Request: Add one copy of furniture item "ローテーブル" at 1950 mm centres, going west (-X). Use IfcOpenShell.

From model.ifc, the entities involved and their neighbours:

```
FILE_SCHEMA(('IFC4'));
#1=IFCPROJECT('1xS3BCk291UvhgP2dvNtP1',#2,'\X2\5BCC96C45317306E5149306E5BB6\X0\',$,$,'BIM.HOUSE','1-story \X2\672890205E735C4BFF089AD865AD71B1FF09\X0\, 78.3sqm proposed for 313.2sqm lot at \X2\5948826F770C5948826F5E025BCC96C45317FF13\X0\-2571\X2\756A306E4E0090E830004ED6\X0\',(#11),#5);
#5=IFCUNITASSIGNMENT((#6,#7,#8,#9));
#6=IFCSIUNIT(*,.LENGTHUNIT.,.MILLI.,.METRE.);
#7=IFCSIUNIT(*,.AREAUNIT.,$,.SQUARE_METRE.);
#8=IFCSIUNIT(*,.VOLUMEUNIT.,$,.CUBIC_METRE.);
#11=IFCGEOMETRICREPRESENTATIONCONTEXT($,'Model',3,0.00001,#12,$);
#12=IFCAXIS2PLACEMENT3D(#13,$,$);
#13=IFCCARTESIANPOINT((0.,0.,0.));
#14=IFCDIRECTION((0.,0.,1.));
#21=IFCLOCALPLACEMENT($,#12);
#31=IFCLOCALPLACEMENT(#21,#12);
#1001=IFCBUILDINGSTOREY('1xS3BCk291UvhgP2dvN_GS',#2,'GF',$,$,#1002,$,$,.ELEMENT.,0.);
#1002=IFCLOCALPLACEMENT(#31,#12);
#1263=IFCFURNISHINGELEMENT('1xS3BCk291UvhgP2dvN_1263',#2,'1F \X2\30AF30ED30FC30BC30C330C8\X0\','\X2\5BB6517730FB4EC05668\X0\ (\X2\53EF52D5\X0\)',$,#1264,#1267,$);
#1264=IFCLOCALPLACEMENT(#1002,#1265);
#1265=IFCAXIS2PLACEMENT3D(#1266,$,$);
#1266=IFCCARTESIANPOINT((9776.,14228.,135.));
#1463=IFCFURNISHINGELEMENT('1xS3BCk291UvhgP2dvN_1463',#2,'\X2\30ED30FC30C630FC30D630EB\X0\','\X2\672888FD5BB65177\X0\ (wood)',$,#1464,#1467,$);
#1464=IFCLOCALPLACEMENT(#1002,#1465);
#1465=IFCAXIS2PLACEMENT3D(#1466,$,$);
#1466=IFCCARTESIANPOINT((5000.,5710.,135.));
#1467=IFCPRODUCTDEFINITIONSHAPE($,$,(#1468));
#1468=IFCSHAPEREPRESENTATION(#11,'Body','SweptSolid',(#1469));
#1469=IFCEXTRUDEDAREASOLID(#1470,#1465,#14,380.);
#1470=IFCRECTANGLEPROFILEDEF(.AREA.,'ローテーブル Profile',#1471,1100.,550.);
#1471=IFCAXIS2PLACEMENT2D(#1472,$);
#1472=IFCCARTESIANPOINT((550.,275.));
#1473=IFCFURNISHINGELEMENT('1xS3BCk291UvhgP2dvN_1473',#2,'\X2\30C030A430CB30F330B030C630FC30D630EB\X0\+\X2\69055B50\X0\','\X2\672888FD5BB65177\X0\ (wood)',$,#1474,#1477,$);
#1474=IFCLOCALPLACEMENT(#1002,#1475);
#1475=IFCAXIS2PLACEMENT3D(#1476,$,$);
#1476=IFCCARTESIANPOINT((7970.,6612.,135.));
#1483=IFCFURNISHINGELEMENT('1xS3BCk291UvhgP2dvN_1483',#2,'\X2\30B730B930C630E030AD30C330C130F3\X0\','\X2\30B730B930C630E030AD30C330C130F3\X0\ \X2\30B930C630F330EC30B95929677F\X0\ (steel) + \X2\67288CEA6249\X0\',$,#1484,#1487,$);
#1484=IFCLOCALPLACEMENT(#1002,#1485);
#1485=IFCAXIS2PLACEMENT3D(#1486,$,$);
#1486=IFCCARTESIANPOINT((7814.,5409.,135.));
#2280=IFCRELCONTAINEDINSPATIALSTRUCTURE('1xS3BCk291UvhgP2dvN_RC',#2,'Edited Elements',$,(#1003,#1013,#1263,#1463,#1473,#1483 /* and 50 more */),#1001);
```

```python
import numpy as np
import ifcopenshell
import ifcopenshell.api.geometry
import ifcopenshell.api.root
import ifcopenshell.util.element
import ifcopenshell.util.placement
import ifcopenshell.util.unit

model = ifcopenshell.open("model.ifc")
unit_scale = ifcopenshell.util.unit.calculate_unit_scale(model)


def reuse_history(source, copy):
    """copy_class also copies each property set's owner history, people and application; keep the originals."""
    for rel in copy.IsDefinedBy:
        if rel.is_a("IfcRelDefinesByProperties") and (history := rel.RelatingPropertyDefinition.OwnerHistory):
            rel.RelatingPropertyDefinition.OwnerHistory = source.OwnerHistory
            ifcopenshell.util.element.remove_deep2(model, history)


source = model.by_guid("1xS3BCk291UvhgP2dvN_1463")
base = ifcopenshell.util.placement.get_local_placement(source.ObjectPlacement)
step = np.array([-1.0, 0.0, 0.0]) * 1.95 / unit_scale

for i in range(1, 2):
    copy = ifcopenshell.api.root.copy_class(model, product=source)
    copy.Representation = ifcopenshell.util.element.copy_deep(
        model, source.Representation, exclude=["IfcGeometricRepresentationContext", "IfcRepresentationMap"]
    )
    reuse_history(source, copy)
    matrix = base.copy()
    matrix[:3, 3] += i * step
    print("added at", matrix[:3, 3].round(3) + 0.0)
    ifcopenshell.api.geometry.edit_object_placement(model, product=copy, matrix=matrix, is_si=False)

model.write("model_updated.ifc")
```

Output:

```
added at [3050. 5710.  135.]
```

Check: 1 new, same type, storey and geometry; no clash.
